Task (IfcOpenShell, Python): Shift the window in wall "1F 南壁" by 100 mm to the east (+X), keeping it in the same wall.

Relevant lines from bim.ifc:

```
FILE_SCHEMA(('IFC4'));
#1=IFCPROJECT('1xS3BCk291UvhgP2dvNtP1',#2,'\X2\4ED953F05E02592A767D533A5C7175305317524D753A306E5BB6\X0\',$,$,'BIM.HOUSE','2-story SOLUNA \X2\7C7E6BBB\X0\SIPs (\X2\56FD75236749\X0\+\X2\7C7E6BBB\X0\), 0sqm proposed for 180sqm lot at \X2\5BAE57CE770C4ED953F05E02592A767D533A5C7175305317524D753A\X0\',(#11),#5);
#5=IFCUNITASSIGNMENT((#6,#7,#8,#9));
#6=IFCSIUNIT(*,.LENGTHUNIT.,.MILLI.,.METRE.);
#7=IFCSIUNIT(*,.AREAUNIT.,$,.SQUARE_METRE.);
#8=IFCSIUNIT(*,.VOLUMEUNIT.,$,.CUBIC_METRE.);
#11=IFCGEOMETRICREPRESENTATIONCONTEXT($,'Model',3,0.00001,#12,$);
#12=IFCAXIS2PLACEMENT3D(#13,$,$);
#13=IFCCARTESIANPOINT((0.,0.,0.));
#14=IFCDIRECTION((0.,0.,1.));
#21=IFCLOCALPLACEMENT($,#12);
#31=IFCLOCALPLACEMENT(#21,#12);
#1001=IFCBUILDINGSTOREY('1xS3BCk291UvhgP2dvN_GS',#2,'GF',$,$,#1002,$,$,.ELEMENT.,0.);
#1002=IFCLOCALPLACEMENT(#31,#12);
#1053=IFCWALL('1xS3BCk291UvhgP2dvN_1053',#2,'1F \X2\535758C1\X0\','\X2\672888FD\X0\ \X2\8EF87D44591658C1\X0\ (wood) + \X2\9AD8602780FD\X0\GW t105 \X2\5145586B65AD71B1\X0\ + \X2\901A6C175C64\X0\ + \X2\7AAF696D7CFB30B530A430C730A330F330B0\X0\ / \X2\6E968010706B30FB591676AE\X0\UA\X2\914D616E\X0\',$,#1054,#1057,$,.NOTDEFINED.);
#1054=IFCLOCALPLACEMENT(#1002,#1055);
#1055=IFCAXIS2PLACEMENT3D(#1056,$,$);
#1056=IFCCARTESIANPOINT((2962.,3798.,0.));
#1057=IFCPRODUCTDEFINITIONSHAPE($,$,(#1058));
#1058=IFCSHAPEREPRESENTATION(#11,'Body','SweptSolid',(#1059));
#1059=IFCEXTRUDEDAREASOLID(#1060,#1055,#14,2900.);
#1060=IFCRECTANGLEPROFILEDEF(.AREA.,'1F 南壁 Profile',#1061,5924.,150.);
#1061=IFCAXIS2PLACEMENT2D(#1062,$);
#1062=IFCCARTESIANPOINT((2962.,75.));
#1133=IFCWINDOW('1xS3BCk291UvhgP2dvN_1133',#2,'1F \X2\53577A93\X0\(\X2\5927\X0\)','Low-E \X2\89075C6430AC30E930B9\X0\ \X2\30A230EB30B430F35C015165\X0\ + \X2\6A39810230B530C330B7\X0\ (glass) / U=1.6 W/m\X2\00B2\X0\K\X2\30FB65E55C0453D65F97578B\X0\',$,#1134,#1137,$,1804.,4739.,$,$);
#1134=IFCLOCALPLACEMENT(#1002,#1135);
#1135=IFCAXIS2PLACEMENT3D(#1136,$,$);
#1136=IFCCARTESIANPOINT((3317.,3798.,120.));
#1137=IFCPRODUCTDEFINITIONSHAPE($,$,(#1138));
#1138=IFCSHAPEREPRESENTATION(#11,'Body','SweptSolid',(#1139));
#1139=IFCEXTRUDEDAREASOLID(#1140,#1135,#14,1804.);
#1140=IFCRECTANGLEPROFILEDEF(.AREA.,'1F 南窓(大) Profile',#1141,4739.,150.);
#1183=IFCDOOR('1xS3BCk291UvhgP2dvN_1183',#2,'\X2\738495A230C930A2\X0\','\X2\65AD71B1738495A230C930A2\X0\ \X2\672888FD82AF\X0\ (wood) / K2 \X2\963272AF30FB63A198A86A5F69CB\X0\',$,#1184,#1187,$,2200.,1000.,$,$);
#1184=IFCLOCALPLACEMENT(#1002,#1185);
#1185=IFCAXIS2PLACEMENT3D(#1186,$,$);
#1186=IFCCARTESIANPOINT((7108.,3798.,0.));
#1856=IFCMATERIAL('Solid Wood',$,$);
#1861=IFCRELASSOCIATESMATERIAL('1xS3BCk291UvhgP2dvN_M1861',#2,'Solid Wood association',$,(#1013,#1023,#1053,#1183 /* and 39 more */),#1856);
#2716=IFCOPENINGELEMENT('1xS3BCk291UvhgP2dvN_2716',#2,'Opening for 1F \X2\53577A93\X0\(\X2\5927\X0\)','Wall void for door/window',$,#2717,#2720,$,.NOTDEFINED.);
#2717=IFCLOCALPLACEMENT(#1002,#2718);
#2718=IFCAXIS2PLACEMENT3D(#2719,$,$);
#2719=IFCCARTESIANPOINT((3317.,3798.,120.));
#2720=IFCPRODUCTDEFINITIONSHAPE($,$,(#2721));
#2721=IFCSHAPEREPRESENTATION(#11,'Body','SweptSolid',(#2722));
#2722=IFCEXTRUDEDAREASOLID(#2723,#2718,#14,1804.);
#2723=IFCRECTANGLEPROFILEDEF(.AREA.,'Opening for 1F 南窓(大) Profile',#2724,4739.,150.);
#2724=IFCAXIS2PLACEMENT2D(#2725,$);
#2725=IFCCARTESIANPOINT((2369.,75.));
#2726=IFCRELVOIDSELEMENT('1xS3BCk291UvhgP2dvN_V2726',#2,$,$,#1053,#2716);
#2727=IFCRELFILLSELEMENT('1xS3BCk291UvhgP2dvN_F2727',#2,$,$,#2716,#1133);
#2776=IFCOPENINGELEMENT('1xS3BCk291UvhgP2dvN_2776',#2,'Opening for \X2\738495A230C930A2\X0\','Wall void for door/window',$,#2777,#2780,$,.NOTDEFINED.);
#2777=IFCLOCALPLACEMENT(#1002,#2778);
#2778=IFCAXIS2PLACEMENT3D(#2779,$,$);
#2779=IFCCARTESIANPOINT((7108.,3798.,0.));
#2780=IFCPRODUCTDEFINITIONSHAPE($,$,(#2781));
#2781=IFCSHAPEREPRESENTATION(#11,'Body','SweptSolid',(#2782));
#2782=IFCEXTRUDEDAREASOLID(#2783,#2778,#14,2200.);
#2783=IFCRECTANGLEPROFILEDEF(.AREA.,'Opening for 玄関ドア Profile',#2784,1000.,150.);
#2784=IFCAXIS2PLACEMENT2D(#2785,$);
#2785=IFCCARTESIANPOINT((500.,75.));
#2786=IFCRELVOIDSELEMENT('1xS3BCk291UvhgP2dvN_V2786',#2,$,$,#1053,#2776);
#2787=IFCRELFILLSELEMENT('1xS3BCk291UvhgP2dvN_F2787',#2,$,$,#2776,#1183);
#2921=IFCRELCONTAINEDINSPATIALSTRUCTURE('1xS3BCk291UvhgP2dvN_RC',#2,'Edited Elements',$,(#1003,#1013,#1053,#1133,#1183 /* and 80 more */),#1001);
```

```python
import ifcopenshell
import ifcopenshell.api.geometry
import ifcopenshell.util.placement

model = ifcopenshell.open("bim.ifc")

window = model.by_guid("1xS3BCk291UvhgP2dvN_1133")
opening = window.FillsVoids[0].RelatingOpeningElement
wall = opening.VoidsElements[0].RelatingBuildingElement

wall_matrix = ifcopenshell.util.placement.get_local_placement(wall.ObjectPlacement)
shift = wall_matrix[:3, 0] * 100.0
before = ifcopenshell.util.placement.get_local_placement(window.ObjectPlacement)[:3, 3].copy()

# The window is not placed relative to its opening, so move both.
for product in (opening, window):
    matrix = ifcopenshell.util.placement.get_local_placement(product.ObjectPlacement)
    matrix[:3, 3] += shift
    ifcopenshell.api.geometry.edit_object_placement(model, product=product, matrix=matrix, is_si=False)

after = ifcopenshell.util.placement.get_local_placement(window.ObjectPlacement)[:3, 3]
print("window moved by", (after - before).round(3) + 0.0)

model.write("bim-out.ifc")
```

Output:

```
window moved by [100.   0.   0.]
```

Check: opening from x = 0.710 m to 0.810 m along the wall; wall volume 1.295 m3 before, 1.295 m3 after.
